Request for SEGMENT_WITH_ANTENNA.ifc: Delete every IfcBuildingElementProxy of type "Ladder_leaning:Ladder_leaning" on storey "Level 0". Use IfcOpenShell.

First a look at what the model holds.

```python
import ifcopenshell
import ifcopenshell.util.element

model = ifcopenshell.open("SEGMENT_WITH_ANTENNA.ifc")
print(model.schema)
storey = next(s for s in model.by_type("IfcBuildingStorey") if s.Name == "Level 0")
proxies = [e for e in ifcopenshell.util.element.get_decomposition(storey) if e.is_a("IfcBuildingElementProxy")]
seen = {}
for e in proxies:
    element_type = ifcopenshell.util.element.get_type(e)
    name = element_type.Name if element_type not in (None, e) else None
    seen[name] = seen.get(name, 0) + 1
for name, count in sorted(seen.items(), key=str):
    print(count, "x", name)
```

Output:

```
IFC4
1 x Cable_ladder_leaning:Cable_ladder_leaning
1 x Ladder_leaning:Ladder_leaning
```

```python
import ifcopenshell
import ifcopenshell.api.root
import ifcopenshell.util.element

model = ifcopenshell.open("SEGMENT_WITH_ANTENNA.ifc")

storey = next(s for s in model.by_type("IfcBuildingStorey") if s.Name == "Level 0")
proxies = [e for e in ifcopenshell.util.element.get_decomposition(storey) if e.is_a("IfcBuildingElementProxy")]
targets = [e for e in proxies if (t := ifcopenshell.util.element.get_type(e)) not in (None, e) and t.Name == "Ladder_leaning:Ladder_leaning"]

for e in targets:
    ifcopenshell.api.root.remove_product(model, product=e)
print(len(targets), "removed")

model.write("SEGMENT_WITH_ANTENNA_v2.ifc")
```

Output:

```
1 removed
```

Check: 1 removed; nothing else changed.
